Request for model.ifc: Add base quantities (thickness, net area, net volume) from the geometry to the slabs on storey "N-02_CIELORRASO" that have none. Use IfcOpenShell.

First a look at what the model holds.

```python
import ifcopenshell
import ifcopenshell.util.element
import ifcopenshell.util.unit

model = ifcopenshell.open("model.ifc")
print(model.schema)
for unit_type in ("LENGTHUNIT", "AREAUNIT", "VOLUMEUNIT"):
    print(unit_type, ifcopenshell.util.unit.calculate_unit_scale(model, unit_type))
storey = next(s for s in model.by_type("IfcBuildingStorey") if s.Name == "N-02_CIELORRASO")
slabs = [e for e in ifcopenshell.util.element.get_decomposition(storey) if e.is_a("IfcSlab")]
for e in sorted(slabs, key=lambda e: e.id()):
    print(e.id(), e.is_a(), e.Name, list(ifcopenshell.util.element.get_psets(e, qtos_only=True)), sep=" | ")
```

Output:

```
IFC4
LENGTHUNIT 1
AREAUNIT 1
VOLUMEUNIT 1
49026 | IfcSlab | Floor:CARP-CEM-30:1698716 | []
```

```python
import ifcopenshell
import ifcopenshell.api.pset
import ifcopenshell.geom
import ifcopenshell.util.element
import ifcopenshell.util.shape
import ifcopenshell.util.unit

model = ifcopenshell.open("model.ifc")
unit_scale = ifcopenshell.util.unit.calculate_unit_scale(model)
area_scale = ifcopenshell.util.unit.calculate_unit_scale(model, "AREAUNIT")
volume_scale = ifcopenshell.util.unit.calculate_unit_scale(model, "VOLUMEUNIT")
settings = ifcopenshell.geom.settings()

storey = next(s for s in model.by_type("IfcBuildingStorey") if s.Name == "N-02_CIELORRASO")
slabs = [e for e in ifcopenshell.util.element.get_decomposition(storey) if e.is_a("IfcSlab")]

for e in sorted(slabs, key=lambda e: e.id()):
    if ifcopenshell.util.element.get_psets(e, qtos_only=True, should_inherit=False):
        continue
    # Geometry comes back in metres, in the element's own axes.
    shape = ifcopenshell.geom.create_shape(settings, e)
    values = {
        "Width": ifcopenshell.util.shape.get_z(shape.geometry) / unit_scale,
        "NetArea": ifcopenshell.util.shape.get_footprint_area(shape.geometry) / area_scale,
        "NetVolume": ifcopenshell.util.shape.get_volume(shape.geometry) / volume_scale,
    }
    qto = ifcopenshell.api.pset.add_qto(model, product=e, name="Qto_SlabBaseQuantities")
    ifcopenshell.api.pset.edit_qto(model, qto=qto, properties=values)
    print(e.id(), {k: round(v, 3) for k, v in values.items()})

model.write("model_rev.ifc")
```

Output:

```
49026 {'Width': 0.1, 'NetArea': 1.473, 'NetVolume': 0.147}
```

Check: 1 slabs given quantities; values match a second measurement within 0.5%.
